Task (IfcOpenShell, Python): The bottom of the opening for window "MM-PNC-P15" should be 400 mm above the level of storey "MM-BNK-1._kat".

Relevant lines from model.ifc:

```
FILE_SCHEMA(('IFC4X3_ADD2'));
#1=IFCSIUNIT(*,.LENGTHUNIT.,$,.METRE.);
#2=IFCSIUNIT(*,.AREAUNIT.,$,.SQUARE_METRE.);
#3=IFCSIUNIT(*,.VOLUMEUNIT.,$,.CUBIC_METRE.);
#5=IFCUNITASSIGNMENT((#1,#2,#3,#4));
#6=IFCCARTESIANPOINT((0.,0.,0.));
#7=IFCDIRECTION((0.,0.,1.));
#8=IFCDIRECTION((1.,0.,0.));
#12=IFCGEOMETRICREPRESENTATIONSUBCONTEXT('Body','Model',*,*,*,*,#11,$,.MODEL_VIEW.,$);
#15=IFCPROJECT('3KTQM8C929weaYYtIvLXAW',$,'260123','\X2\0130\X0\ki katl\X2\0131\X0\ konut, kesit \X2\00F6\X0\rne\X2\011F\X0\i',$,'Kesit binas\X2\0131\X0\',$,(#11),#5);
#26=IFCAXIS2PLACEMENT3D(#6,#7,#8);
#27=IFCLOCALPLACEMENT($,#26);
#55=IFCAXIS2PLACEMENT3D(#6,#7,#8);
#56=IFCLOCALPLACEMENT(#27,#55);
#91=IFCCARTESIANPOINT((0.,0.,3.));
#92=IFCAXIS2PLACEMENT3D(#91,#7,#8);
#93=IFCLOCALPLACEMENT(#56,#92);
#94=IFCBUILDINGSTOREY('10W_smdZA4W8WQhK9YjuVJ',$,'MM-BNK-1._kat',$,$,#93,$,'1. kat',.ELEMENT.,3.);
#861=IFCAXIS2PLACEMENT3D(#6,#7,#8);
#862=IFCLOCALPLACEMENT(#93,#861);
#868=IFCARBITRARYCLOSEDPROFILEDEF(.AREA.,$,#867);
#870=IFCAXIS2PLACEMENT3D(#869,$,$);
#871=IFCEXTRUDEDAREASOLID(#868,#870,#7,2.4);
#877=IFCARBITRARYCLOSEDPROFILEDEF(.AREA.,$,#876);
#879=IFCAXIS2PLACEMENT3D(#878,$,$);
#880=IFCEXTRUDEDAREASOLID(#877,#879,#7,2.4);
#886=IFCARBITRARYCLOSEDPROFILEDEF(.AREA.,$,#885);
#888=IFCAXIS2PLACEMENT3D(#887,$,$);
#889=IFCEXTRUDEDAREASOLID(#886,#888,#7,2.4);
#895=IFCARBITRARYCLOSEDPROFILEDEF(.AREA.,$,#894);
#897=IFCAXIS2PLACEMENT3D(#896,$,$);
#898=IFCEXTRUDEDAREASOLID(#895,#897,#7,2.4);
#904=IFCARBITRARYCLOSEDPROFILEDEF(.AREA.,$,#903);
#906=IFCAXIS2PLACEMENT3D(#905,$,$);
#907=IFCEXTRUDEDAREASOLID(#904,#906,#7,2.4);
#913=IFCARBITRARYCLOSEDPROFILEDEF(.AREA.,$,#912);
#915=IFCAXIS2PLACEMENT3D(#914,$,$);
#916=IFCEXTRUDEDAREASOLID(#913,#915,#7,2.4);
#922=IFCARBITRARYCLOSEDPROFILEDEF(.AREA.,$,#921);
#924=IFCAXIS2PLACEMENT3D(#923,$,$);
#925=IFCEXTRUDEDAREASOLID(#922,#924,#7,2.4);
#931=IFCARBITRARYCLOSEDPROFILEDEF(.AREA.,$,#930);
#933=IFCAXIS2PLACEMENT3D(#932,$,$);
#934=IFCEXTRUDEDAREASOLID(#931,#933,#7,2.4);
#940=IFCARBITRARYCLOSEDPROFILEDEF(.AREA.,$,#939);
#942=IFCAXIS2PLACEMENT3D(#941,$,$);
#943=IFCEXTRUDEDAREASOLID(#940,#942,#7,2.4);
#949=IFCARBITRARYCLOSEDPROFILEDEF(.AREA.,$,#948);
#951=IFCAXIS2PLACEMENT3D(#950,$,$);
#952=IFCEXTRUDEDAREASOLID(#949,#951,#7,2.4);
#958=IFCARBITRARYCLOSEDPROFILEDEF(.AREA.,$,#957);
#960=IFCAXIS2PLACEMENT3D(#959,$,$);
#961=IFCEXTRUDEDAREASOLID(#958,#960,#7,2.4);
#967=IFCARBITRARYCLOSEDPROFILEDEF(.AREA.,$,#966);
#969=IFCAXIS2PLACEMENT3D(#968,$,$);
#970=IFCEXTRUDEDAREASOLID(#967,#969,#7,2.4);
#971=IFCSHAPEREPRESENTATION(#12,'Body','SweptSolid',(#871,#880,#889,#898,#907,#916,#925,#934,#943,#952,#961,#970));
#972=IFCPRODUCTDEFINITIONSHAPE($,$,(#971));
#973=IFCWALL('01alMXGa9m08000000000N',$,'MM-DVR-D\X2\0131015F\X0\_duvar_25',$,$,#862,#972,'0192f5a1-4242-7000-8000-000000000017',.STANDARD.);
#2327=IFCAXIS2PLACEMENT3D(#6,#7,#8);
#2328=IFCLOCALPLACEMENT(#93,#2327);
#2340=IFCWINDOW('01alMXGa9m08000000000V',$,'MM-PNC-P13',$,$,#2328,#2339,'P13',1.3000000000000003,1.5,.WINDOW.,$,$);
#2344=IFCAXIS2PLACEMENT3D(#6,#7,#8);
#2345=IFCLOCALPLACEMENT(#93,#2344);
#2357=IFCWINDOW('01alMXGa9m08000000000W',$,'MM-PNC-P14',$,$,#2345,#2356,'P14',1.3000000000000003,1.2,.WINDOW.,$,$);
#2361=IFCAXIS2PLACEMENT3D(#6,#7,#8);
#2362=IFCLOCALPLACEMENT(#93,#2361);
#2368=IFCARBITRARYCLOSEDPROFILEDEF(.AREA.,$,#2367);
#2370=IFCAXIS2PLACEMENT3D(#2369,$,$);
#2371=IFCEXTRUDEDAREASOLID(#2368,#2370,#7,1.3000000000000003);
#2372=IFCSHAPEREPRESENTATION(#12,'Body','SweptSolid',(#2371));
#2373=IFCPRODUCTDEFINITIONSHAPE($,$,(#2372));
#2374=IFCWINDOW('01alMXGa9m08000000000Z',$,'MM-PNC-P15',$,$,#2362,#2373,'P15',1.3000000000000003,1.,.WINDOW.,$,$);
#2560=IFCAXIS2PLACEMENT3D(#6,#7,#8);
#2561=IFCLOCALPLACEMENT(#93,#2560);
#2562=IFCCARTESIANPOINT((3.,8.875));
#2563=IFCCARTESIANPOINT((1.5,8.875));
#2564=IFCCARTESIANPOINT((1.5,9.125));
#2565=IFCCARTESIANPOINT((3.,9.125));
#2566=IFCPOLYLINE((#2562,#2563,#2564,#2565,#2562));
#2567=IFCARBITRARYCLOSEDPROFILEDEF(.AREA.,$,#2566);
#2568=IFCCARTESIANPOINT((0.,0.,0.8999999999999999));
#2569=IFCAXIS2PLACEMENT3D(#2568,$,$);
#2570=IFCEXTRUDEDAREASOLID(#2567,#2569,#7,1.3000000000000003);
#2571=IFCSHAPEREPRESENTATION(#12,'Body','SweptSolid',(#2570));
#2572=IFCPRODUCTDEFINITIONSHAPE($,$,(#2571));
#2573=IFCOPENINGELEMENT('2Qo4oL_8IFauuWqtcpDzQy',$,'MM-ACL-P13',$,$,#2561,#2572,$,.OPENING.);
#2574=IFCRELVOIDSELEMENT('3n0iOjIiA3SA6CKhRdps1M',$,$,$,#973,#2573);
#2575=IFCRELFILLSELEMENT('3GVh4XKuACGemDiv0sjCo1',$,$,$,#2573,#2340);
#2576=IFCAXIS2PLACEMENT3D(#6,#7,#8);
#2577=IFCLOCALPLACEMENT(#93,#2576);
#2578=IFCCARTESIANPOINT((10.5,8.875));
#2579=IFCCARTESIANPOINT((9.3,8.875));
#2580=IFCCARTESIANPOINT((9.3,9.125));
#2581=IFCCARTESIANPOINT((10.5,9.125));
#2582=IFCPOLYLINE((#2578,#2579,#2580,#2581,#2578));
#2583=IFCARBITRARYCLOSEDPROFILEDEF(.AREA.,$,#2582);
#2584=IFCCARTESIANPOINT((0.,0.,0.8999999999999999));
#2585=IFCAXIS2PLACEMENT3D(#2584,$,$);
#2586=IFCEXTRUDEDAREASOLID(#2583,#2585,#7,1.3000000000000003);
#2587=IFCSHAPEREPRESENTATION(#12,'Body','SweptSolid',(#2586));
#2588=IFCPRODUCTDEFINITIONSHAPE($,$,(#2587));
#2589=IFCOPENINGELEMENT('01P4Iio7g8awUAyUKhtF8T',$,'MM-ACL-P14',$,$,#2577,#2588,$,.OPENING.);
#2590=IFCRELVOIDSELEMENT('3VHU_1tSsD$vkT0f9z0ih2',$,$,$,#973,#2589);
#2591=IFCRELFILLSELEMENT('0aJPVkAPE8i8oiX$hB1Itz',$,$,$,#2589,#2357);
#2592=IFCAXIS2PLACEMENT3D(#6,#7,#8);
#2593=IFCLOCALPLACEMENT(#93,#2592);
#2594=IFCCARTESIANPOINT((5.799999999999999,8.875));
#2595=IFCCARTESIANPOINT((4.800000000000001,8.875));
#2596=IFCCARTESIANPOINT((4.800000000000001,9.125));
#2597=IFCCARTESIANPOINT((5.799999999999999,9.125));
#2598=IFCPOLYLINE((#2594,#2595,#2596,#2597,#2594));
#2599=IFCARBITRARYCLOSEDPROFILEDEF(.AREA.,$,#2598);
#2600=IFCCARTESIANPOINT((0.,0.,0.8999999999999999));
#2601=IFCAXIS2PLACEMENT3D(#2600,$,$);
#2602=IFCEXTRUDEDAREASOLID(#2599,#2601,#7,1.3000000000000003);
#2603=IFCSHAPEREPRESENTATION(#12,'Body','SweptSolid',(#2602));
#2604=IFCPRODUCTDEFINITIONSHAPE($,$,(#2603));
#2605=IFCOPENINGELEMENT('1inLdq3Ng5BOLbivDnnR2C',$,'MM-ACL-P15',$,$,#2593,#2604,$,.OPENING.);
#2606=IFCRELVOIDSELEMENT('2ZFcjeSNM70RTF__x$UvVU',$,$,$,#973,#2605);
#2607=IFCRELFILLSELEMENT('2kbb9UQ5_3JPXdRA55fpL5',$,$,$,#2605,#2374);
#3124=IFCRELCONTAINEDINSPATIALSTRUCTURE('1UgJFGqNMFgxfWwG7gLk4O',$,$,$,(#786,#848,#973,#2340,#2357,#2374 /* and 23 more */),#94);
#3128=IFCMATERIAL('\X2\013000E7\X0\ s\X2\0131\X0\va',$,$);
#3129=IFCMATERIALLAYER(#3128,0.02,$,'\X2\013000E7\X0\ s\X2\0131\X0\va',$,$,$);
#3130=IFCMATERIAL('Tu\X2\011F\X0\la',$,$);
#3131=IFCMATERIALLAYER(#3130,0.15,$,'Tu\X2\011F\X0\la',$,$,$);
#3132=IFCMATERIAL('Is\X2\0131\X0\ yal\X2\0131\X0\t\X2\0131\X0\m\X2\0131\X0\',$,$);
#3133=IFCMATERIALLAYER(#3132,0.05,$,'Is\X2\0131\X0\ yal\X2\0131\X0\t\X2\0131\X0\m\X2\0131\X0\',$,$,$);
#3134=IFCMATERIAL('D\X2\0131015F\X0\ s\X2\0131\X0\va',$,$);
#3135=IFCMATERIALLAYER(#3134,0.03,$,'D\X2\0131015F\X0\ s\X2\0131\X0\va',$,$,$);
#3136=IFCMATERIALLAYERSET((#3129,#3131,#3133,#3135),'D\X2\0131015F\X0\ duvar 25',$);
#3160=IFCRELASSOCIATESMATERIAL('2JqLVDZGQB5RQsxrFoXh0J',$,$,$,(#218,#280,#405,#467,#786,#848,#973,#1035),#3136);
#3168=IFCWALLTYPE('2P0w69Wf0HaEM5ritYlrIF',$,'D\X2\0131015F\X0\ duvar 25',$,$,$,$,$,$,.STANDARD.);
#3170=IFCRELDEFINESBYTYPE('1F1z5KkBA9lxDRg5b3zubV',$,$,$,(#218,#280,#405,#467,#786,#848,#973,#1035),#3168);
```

```python
import numpy as np
import ifcopenshell
import ifcopenshell.api.geometry
import ifcopenshell.geom
import ifcopenshell.util.element
import ifcopenshell.util.placement
import ifcopenshell.util.shape
import ifcopenshell.util.unit

model = ifcopenshell.open("model.ifc")
unit_scale = ifcopenshell.util.unit.calculate_unit_scale(model)

window = model.by_guid("01alMXGa9m08000000000Z")
opening = window.FillsVoids[0].RelatingOpeningElement
storey = ifcopenshell.util.element.get_container(window, ifc_class="IfcBuildingStorey")
level = ifcopenshell.util.placement.get_local_placement(storey.ObjectPlacement)[2, 3]

# The opening's origin need not be at the sill, so measure its lowest point.
shape = ifcopenshell.geom.create_shape(ifcopenshell.geom.settings(), opening)
bottom = ifcopenshell.util.shape.get_shape_bottom_elevation(shape, shape.geometry) / unit_scale
dz = level + 0.4 - bottom

shift = np.array([0.0, 0.0, dz])
# The window is not placed relative to its opening, so move both.
for product in (opening, window):
    matrix = ifcopenshell.util.placement.get_local_placement(product.ObjectPlacement)
    matrix[:3, 3] += shift
    ifcopenshell.api.geometry.edit_object_placement(model, product=product, matrix=matrix, is_si=False)

print(f"moved by {dz * unit_scale:+.3f} m")

model.write("model-out.ifc")
```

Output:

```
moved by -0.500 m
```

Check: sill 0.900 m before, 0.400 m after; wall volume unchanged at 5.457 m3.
